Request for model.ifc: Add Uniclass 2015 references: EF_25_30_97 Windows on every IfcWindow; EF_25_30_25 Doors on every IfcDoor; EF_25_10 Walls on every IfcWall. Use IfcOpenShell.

First a look at what the model holds.

```python
import ifcopenshell

model = ifcopenshell.open("model.ifc")
print(model.schema)
print("classifications:", [c.Name for c in model.by_type("IfcClassification")])
for ifc_class in ("IfcDoor", "IfcRoof", "IfcStair", "IfcWall", "IfcWindow"):
    print(ifc_class, len(model.by_type(ifc_class)))
```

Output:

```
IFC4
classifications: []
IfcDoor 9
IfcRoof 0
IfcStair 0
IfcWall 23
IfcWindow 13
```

```python
import ifcopenshell
import ifcopenshell.api.classification

model = ifcopenshell.open("model.ifc")

system = ifcopenshell.api.classification.add_classification(model, classification="Uniclass 2015")

codes = {
    "IfcWindow": ("EF_25_30_97", "Windows"),
    "IfcDoor": ("EF_25_30_25", "Doors"),
    "IfcWall": ("EF_25_10", "Walls"),
}
for ifc_class, (code, name) in codes.items():
    products = model.by_type(ifc_class)
    ifcopenshell.api.classification.add_reference(
        model, products=products, classification=system, identification=code, name=name
    )
    print(code, len(products))

model.write("model_v2.ifc")
```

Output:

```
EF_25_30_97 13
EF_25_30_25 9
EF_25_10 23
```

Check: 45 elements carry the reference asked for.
